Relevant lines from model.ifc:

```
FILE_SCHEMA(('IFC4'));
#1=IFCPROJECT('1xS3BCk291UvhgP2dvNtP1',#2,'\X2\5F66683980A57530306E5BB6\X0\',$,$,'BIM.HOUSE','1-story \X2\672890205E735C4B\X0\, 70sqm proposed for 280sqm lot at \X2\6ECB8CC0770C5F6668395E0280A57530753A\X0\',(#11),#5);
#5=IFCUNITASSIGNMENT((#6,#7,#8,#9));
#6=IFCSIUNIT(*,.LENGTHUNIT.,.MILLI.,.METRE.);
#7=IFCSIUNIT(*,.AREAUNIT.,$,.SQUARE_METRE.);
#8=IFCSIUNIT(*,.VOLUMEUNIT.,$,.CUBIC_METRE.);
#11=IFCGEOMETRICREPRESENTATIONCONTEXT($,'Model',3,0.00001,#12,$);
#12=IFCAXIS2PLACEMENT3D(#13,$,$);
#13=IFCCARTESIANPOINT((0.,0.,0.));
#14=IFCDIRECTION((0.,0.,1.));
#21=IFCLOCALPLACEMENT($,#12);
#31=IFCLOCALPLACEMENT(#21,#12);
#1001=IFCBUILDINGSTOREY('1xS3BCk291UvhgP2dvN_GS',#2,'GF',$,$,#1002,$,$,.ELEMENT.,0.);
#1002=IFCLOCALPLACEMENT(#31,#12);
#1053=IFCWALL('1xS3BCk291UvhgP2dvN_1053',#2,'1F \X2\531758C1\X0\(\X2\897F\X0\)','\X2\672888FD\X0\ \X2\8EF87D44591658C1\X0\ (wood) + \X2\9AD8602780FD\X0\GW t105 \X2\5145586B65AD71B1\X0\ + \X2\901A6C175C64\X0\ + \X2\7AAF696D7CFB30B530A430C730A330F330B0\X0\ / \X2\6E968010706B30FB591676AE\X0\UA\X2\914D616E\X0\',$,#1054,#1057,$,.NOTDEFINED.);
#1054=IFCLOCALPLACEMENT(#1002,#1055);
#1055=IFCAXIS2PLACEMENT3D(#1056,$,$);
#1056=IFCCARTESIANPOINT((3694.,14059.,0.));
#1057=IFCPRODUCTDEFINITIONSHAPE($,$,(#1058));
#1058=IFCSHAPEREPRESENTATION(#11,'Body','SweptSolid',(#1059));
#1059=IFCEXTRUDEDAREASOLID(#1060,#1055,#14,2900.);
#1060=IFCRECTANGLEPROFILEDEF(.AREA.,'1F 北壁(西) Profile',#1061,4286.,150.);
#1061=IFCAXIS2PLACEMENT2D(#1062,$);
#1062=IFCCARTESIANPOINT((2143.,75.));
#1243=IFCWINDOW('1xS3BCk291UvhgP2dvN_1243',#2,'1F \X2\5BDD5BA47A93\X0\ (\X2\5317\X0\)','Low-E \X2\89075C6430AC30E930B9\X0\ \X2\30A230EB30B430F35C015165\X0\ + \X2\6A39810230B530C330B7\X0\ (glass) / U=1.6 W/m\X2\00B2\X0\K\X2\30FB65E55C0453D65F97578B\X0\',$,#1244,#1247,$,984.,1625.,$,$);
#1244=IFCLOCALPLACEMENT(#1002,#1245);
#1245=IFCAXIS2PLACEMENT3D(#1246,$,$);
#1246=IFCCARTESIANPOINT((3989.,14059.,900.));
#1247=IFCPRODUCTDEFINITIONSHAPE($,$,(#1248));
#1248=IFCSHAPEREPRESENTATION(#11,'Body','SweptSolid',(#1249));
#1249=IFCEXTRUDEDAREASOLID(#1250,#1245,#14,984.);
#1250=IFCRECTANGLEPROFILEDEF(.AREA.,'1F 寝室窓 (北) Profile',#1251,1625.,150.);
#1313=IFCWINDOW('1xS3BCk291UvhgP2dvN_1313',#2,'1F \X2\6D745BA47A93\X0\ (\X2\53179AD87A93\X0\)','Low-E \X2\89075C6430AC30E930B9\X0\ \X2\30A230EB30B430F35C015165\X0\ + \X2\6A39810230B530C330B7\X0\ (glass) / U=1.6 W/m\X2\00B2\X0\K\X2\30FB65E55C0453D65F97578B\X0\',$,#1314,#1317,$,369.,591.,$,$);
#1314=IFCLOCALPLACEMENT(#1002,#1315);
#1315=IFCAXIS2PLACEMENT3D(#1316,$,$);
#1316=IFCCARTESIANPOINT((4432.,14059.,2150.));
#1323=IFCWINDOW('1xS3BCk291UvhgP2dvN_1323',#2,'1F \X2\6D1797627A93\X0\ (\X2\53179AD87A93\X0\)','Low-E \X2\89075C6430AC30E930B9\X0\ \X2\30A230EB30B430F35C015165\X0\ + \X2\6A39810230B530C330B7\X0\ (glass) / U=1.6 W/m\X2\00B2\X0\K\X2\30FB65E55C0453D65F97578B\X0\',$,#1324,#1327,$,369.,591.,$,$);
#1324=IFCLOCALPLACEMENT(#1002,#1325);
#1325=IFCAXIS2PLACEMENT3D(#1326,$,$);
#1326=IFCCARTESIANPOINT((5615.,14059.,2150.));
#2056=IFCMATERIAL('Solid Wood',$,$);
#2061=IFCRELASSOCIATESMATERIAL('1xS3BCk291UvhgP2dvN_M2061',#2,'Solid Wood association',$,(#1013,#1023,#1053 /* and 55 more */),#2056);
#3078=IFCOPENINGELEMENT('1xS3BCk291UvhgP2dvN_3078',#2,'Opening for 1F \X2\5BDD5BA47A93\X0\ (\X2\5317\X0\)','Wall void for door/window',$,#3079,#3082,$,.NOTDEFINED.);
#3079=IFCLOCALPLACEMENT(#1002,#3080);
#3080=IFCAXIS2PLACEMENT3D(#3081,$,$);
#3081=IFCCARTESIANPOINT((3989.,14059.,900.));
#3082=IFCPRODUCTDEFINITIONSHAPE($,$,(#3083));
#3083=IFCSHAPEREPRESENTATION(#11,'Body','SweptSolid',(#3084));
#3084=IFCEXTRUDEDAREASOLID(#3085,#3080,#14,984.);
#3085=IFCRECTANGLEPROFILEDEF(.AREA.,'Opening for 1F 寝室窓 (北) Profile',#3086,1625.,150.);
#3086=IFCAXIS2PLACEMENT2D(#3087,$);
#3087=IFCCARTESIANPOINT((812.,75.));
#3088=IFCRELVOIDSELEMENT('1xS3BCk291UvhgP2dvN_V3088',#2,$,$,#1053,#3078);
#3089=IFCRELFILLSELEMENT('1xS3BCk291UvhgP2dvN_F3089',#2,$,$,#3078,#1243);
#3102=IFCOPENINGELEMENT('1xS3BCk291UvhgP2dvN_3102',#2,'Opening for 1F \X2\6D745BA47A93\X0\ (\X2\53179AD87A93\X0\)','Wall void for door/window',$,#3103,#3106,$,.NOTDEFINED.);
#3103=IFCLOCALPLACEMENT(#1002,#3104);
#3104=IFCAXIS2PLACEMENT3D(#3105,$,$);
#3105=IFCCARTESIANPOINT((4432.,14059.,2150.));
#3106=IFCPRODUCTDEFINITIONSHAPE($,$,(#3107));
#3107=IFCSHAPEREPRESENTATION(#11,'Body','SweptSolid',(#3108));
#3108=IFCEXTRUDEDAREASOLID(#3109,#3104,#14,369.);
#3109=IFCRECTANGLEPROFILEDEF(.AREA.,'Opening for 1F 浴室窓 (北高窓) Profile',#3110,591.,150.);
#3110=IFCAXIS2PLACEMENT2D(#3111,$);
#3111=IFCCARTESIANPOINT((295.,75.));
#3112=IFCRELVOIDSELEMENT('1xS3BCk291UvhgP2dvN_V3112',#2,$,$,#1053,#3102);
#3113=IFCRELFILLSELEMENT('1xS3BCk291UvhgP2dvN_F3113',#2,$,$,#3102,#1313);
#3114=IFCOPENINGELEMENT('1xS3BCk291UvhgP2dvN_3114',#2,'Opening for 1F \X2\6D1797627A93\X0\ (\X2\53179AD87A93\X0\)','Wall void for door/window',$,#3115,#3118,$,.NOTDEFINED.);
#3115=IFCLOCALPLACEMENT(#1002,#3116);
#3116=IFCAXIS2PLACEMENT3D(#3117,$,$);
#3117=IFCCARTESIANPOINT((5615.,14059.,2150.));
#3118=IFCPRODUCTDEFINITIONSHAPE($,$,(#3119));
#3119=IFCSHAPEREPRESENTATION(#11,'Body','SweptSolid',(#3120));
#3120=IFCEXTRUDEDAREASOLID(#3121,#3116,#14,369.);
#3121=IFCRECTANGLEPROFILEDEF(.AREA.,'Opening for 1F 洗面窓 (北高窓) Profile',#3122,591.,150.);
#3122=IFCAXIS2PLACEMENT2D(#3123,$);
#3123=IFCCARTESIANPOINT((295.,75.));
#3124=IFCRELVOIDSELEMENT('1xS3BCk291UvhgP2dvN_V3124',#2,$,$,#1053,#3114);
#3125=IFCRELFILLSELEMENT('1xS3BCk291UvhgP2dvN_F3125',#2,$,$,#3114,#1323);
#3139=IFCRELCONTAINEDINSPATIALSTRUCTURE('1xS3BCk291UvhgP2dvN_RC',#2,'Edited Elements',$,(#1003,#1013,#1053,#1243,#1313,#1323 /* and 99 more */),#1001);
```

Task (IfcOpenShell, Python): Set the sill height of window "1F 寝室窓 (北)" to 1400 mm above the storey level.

```python
import numpy as np
import ifcopenshell
import ifcopenshell.api.geometry
import ifcopenshell.geom
import ifcopenshell.util.element
import ifcopenshell.util.placement
import ifcopenshell.util.shape
import ifcopenshell.util.unit

model = ifcopenshell.open("model.ifc")
unit_scale = ifcopenshell.util.unit.calculate_unit_scale(model)

window = model.by_guid("1xS3BCk291UvhgP2dvN_1243")
opening = window.FillsVoids[0].RelatingOpeningElement
storey = ifcopenshell.util.element.get_container(window, ifc_class="IfcBuildingStorey")
level = ifcopenshell.util.placement.get_local_placement(storey.ObjectPlacement)[2, 3]

# The opening's origin need not be at the sill, so measure its lowest point.
shape = ifcopenshell.geom.create_shape(ifcopenshell.geom.settings(), opening)
bottom = ifcopenshell.util.shape.get_shape_bottom_elevation(shape, shape.geometry) / unit_scale
dz = level + 1.4 / unit_scale - bottom

shift = np.array([0.0, 0.0, dz])
# The window is not placed relative to its opening, so move both.
for product in (opening, window):
    matrix = ifcopenshell.util.placement.get_local_placement(product.ObjectPlacement)
    matrix[:3, 3] += shift
    ifcopenshell.api.geometry.edit_object_placement(model, product=product, matrix=matrix, is_si=False)

print(f"moved by {dz * unit_scale:+.3f} m")

model.write("model_edited.ifc")
```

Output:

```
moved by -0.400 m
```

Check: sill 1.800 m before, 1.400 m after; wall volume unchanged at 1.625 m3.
